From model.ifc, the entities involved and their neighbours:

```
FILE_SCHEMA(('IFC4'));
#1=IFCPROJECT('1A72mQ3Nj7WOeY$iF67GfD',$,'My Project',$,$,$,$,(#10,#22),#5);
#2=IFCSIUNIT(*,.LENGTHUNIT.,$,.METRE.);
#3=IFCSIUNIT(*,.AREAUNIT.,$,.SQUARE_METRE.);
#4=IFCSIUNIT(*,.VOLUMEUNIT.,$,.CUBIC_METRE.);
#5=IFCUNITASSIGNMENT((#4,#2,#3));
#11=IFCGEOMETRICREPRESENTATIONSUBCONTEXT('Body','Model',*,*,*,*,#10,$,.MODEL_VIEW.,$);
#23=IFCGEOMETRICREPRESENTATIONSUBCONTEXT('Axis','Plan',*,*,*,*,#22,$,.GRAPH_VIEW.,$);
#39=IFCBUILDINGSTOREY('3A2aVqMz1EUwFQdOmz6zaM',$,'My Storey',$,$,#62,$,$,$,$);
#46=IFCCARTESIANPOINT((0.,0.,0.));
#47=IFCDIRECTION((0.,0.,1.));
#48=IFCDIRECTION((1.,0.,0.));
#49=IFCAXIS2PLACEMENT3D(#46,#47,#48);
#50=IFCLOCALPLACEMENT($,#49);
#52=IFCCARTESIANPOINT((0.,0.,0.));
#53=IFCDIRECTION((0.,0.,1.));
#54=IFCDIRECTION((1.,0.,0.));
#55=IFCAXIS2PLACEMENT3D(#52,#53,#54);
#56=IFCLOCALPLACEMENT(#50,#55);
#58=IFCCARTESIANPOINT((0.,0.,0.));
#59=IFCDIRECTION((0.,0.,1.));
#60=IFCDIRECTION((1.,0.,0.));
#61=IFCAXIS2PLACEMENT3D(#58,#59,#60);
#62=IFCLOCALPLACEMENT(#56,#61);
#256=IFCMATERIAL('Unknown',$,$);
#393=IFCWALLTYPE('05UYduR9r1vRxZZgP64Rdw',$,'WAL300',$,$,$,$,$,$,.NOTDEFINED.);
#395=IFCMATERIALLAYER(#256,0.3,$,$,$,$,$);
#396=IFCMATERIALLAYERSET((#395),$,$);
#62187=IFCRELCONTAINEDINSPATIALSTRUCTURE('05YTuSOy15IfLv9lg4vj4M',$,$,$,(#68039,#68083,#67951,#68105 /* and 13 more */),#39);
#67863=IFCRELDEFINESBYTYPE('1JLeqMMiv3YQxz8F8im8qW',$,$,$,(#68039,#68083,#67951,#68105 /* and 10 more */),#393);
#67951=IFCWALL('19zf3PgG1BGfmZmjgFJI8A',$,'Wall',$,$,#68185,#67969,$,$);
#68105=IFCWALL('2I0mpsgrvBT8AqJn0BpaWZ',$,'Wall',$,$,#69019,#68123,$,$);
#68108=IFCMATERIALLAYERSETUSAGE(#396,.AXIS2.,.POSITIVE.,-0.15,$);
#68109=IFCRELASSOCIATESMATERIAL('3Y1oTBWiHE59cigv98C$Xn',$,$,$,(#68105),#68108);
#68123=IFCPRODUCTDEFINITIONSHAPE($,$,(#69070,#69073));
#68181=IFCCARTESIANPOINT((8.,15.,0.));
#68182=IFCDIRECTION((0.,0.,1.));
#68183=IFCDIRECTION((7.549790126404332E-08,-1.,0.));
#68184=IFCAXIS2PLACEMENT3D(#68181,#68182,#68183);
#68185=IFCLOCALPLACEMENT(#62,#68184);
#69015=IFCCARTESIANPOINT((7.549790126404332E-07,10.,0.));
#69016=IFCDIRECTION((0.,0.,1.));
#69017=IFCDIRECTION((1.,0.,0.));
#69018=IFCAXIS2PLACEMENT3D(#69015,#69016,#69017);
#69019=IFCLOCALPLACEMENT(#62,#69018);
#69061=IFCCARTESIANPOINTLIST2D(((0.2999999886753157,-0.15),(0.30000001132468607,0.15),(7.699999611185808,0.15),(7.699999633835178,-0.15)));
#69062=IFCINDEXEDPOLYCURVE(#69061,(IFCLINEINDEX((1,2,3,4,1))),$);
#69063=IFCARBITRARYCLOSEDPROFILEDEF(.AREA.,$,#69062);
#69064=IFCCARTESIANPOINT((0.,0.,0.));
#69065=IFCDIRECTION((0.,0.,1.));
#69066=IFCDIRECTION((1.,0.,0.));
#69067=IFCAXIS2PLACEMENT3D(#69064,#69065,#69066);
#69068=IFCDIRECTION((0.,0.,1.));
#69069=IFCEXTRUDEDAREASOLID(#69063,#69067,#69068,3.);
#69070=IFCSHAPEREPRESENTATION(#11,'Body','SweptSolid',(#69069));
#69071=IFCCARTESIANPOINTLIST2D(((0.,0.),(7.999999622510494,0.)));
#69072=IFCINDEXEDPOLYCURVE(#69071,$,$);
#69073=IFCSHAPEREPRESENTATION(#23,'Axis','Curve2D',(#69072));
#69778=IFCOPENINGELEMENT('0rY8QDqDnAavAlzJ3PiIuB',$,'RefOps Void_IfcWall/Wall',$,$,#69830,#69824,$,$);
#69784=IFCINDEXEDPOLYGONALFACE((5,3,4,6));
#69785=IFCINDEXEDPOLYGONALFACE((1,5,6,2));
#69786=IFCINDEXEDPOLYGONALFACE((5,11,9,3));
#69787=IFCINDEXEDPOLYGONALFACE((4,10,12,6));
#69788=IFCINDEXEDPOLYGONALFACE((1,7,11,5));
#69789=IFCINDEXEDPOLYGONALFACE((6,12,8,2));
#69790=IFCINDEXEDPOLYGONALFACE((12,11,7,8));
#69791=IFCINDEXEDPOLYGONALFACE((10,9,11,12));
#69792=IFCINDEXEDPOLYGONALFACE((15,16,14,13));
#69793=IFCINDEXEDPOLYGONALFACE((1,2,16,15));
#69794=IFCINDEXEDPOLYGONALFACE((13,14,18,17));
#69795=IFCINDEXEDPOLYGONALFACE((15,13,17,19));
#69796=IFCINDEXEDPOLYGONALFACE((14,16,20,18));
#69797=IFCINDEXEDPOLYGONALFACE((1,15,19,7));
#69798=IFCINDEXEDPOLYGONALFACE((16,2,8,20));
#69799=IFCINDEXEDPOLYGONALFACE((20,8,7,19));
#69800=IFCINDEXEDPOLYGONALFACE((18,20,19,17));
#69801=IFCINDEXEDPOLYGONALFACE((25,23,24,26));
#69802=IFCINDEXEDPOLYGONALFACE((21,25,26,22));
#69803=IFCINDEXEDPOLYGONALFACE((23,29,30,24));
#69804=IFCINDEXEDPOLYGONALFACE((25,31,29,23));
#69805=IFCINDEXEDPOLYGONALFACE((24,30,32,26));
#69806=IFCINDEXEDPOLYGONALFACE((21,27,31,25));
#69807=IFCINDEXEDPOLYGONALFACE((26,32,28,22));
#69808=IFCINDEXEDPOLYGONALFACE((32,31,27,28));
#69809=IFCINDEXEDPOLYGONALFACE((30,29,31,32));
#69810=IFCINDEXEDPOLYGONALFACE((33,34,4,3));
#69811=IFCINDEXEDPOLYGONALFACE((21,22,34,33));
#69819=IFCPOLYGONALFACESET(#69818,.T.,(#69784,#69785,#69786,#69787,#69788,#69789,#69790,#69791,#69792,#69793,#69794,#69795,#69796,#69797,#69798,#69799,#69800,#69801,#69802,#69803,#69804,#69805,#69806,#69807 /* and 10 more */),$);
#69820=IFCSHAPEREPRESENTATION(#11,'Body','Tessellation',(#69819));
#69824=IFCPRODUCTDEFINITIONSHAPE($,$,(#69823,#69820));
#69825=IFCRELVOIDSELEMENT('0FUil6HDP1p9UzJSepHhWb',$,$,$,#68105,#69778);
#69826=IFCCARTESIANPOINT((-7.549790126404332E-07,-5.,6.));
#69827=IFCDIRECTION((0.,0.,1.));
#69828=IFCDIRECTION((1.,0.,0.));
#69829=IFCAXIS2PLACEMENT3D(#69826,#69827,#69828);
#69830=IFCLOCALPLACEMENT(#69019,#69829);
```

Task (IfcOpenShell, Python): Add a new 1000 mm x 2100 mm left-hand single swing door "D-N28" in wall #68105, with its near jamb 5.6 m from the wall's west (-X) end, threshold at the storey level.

```python
import numpy as np
import ifcopenshell
import ifcopenshell.api.feature
import ifcopenshell.api.geometry
import ifcopenshell.api.root
import ifcopenshell.api.spatial
import ifcopenshell.geom
import ifcopenshell.util.element
import ifcopenshell.util.placement
import ifcopenshell.util.representation
import ifcopenshell.util.shape
import ifcopenshell.util.unit

model = ifcopenshell.open("model.ifc")
unit_scale = ifcopenshell.util.unit.calculate_unit_scale(model)
settings = ifcopenshell.geom.settings()


def volume(element):
    """Net volume in cubic metres, openings subtracted."""
    shape = ifcopenshell.geom.create_shape(settings, element)
    return ifcopenshell.util.shape.get_volume(shape.geometry)


wall = model.by_id(68105)
storey = ifcopenshell.util.element.get_container(wall, ifc_class="IfcBuildingStorey")
context = ifcopenshell.util.representation.get_context(model, "Model", "Body", "MODEL_VIEW")
before = volume(wall)

width, height, from_end, sill = 1, 2.1, 5.6, 0.0  # metres

# The wall runs along its own X axis, and the end named is its -X end.
wall_shape = ifcopenshell.geom.create_shape(settings, wall)
x, y, z = ifcopenshell.util.shape.get_vertices(wall_shape.geometry).T
start = x.min() + from_end
face, thickness = float(y.min()), float(y.max() - y.min())
wall_matrix = ifcopenshell.util.placement.get_local_placement(wall.ObjectPlacement)
level = ifcopenshell.util.placement.get_local_placement(storey.ObjectPlacement)[2, 3]


def in_wall(x, y):
    """Placement at x, y metres in the wall's axes, at sill height."""
    matrix = wall_matrix.copy()
    matrix[:, 3] = wall_matrix @ np.array([x / unit_scale, y / unit_scale, 0.0, 1.0])
    matrix[2, 3] = level + sill / unit_scale
    return matrix


# Opening: a box that overshoots both wall faces by 50 mm.
opening = ifcopenshell.api.root.create_entity(model, ifc_class="IfcOpeningElement", predefined_type="OPENING")
box = ifcopenshell.api.geometry.add_wall_representation(
    model, context=context, length=width, height=height, thickness=thickness + 0.1
)
ifcopenshell.api.geometry.assign_representation(model, product=opening, representation=box)
ifcopenshell.api.geometry.edit_object_placement(model, product=opening, matrix=in_wall(start, face - 0.05), is_si=False)
ifcopenshell.api.feature.add_feature(model, feature=opening, element=wall)

door = ifcopenshell.api.root.create_entity(model, ifc_class="IfcDoor", name="D-N28", predefined_type="DOOR")
door.OverallWidth, door.OverallHeight = width / unit_scale, height / unit_scale
door.OperationType = "SINGLE_SWING_LEFT"
body = ifcopenshell.api.geometry.add_door_representation(
    model,
    context=context,
    overall_width=door.OverallWidth,
    overall_height=door.OverallHeight,
    operation_type="SINGLE_SWING_LEFT",
    lining_properties={"LiningDepth": thickness / unit_scale, "ThresholdDepth": thickness / unit_scale},
)
ifcopenshell.api.geometry.assign_representation(model, product=door, representation=body)
ifcopenshell.api.spatial.assign_container(model, products=[door], relating_structure=storey)
ifcopenshell.api.feature.add_filling(model, opening=opening, element=door)

# The lining spans the wall, so the door starts at the wall face.
ifcopenshell.api.geometry.edit_object_placement(model, product=door, matrix=in_wall(start, face), is_si=False)

after = volume(wall)

print(f"wall volume {before:.3f} -> {after:.3f} m3")

model.write("model-out.ifc")
```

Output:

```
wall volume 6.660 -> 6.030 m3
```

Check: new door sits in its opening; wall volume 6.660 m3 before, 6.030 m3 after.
